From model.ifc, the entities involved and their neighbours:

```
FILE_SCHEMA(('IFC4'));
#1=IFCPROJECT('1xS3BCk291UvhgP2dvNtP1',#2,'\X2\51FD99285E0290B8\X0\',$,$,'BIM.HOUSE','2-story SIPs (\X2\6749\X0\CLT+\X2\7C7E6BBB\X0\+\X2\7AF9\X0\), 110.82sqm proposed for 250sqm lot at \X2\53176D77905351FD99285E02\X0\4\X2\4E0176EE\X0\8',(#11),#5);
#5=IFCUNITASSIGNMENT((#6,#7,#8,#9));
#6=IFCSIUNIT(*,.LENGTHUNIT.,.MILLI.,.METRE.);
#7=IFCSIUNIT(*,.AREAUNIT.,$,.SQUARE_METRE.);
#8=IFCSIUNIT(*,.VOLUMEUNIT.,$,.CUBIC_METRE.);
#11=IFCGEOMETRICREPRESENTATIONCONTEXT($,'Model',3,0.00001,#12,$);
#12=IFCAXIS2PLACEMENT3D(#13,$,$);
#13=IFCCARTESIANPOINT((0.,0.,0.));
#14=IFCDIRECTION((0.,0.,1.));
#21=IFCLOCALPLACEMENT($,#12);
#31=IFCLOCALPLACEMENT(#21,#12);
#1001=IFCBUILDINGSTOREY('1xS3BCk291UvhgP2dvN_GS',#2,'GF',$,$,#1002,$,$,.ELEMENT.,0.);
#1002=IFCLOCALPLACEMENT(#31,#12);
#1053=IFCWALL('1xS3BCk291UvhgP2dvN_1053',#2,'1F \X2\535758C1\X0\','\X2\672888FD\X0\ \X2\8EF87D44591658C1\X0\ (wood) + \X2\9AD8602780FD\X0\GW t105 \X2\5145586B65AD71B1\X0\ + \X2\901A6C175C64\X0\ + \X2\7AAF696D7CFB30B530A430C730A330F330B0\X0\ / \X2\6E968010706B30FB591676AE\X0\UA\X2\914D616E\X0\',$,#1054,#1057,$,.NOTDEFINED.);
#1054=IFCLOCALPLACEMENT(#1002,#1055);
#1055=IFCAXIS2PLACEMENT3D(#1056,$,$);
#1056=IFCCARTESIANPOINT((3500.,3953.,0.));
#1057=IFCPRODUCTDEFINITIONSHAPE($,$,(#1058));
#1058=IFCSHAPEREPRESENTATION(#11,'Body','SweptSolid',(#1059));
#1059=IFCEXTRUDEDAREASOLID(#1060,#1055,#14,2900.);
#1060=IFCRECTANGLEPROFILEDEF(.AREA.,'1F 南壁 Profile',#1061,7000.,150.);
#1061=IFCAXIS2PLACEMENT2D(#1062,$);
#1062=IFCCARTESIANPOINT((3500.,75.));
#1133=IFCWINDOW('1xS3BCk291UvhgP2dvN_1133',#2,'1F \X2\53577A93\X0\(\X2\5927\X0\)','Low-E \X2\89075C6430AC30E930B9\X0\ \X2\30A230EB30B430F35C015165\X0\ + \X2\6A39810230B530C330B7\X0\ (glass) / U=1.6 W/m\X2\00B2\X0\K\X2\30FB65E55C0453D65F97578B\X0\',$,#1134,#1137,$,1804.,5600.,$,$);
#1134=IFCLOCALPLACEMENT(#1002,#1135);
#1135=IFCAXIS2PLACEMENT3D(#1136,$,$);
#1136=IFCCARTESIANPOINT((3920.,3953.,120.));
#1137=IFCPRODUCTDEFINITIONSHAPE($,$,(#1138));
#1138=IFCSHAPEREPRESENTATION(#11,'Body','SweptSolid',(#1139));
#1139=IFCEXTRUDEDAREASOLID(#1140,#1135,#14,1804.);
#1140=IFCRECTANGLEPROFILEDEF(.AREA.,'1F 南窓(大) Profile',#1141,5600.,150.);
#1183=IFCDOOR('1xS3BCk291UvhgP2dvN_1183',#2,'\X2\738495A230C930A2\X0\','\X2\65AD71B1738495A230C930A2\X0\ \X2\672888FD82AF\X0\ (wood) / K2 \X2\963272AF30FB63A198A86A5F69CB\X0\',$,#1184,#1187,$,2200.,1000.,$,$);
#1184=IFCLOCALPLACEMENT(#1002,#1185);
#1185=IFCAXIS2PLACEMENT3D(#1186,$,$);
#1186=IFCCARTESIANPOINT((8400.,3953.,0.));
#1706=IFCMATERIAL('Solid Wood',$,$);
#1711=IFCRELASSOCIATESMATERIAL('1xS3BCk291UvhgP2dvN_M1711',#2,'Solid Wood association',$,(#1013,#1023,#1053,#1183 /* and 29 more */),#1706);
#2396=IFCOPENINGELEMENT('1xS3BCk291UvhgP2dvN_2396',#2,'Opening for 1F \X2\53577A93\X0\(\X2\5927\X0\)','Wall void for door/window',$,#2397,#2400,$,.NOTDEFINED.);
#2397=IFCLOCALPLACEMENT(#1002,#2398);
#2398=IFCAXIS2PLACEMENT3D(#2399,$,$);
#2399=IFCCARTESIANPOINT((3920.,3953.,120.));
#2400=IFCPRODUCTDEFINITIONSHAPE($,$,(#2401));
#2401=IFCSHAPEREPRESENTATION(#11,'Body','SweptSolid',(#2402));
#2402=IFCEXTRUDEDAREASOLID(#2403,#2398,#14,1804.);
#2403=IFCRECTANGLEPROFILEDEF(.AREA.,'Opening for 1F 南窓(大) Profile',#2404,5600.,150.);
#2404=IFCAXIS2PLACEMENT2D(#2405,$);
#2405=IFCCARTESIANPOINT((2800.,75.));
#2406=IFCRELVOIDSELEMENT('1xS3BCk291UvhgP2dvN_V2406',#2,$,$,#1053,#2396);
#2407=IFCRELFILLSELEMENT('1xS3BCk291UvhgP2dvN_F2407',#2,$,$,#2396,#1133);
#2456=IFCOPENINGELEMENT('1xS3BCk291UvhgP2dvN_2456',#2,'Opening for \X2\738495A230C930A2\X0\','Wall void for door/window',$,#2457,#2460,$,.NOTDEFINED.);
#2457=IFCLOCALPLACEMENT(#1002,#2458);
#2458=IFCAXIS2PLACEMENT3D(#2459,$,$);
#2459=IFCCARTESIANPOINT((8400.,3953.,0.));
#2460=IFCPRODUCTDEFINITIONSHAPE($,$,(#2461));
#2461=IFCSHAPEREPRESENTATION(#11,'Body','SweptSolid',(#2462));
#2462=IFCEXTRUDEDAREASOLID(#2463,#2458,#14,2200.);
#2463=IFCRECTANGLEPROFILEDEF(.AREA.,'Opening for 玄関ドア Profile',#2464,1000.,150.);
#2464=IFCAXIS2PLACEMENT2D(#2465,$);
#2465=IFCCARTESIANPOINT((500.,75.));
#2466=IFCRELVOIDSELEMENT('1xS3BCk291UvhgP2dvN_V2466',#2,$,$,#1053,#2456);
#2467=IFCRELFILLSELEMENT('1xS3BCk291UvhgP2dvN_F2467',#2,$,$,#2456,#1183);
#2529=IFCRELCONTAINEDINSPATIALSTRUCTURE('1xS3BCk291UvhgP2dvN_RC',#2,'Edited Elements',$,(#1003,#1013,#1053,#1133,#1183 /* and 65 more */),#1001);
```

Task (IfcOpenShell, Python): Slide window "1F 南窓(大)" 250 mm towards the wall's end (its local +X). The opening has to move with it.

```python
import ifcopenshell
import ifcopenshell.api.geometry
import ifcopenshell.util.placement

model = ifcopenshell.open("model.ifc")

window = model.by_guid("1xS3BCk291UvhgP2dvN_1133")
opening = window.FillsVoids[0].RelatingOpeningElement
wall = opening.VoidsElements[0].RelatingBuildingElement

wall_matrix = ifcopenshell.util.placement.get_local_placement(wall.ObjectPlacement)
shift = wall_matrix[:3, 0] * 250.0
before = ifcopenshell.util.placement.get_local_placement(window.ObjectPlacement)[:3, 3].copy()

# The window is not placed relative to its opening, so move both.
for product in (opening, window):
    matrix = ifcopenshell.util.placement.get_local_placement(product.ObjectPlacement)
    matrix[:3, 3] += shift
    ifcopenshell.api.geometry.edit_object_placement(model, product=product, matrix=matrix, is_si=False)

after = ifcopenshell.util.placement.get_local_placement(window.ObjectPlacement)[:3, 3]
print("window moved by", (after - before).round(3) + 0.0)

model.write("model-out.ifc")
```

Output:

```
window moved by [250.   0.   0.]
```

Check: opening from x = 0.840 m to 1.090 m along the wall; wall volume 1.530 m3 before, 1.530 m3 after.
